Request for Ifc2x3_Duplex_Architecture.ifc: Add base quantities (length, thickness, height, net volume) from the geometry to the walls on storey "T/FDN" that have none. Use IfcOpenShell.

First a look at what the model holds.

```python
import ifcopenshell
import ifcopenshell.util.element
import ifcopenshell.util.unit

model = ifcopenshell.open("Ifc2x3_Duplex_Architecture.ifc")
print(model.schema)
for unit_type in ("LENGTHUNIT", "AREAUNIT", "VOLUMEUNIT"):
    print(unit_type, ifcopenshell.util.unit.calculate_unit_scale(model, unit_type))
storey = next(s for s in model.by_type("IfcBuildingStorey") if s.Name == "T/FDN")
walls = [e for e in ifcopenshell.util.element.get_decomposition(storey) if e.is_a("IfcWall")]
for e in sorted(walls, key=lambda e: e.id()):
    print(e.id(), e.is_a(), e.Name, list(ifcopenshell.util.element.get_psets(e, qtos_only=True)), sep=" | ")
```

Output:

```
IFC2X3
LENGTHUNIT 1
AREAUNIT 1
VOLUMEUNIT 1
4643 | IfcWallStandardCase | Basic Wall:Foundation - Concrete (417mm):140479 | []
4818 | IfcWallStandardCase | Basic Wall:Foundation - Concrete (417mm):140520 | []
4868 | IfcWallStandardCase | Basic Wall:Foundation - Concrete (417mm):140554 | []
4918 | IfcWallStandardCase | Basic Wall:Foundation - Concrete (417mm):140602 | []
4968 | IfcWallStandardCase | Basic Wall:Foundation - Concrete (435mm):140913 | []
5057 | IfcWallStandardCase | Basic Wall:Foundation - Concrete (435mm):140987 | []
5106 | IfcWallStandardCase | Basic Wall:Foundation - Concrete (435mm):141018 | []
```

```python
import ifcopenshell
import ifcopenshell.api.pset
import ifcopenshell.geom
import ifcopenshell.util.element
import ifcopenshell.util.shape
import ifcopenshell.util.unit

model = ifcopenshell.open("Ifc2x3_Duplex_Architecture.ifc")
unit_scale = ifcopenshell.util.unit.calculate_unit_scale(model)
volume_scale = ifcopenshell.util.unit.calculate_unit_scale(model, "VOLUMEUNIT")
settings = ifcopenshell.geom.settings()

storey = next(s for s in model.by_type("IfcBuildingStorey") if s.Name == "T/FDN")
walls = [e for e in ifcopenshell.util.element.get_decomposition(storey) if e.is_a("IfcWall")]

for e in sorted(walls, key=lambda e: e.id()):
    if ifcopenshell.util.element.get_psets(e, qtos_only=True, should_inherit=False):
        continue
    # Geometry comes back in metres, in the element's own axes.
    shape = ifcopenshell.geom.create_shape(settings, e)
    values = {
        "Length": ifcopenshell.util.shape.get_x(shape.geometry) / unit_scale,
        "Width": ifcopenshell.util.shape.get_y(shape.geometry) / unit_scale,
        "Height": ifcopenshell.util.shape.get_z(shape.geometry) / unit_scale,
        "NetVolume": ifcopenshell.util.shape.get_volume(shape.geometry) / volume_scale,
    }
    qto = ifcopenshell.api.pset.add_qto(model, product=e, name="BaseQuantities")
    ifcopenshell.api.pset.edit_qto(model, qto=qto, properties=values)
    print(e.id(), {k: round(v, 3) for k, v in values.items()})

model.write("Ifc2x3_Duplex_Architecture_rev.ifc")
```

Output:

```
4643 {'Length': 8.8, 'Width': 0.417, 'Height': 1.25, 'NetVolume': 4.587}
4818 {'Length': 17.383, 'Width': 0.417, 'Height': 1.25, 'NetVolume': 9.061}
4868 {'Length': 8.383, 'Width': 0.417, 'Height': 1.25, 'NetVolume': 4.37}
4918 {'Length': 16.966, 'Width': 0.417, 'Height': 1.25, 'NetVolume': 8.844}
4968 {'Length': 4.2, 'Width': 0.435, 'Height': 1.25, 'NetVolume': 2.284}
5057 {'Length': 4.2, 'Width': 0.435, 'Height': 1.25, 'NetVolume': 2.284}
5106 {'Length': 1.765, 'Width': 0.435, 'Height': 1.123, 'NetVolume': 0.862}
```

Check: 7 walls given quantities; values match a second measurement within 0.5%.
